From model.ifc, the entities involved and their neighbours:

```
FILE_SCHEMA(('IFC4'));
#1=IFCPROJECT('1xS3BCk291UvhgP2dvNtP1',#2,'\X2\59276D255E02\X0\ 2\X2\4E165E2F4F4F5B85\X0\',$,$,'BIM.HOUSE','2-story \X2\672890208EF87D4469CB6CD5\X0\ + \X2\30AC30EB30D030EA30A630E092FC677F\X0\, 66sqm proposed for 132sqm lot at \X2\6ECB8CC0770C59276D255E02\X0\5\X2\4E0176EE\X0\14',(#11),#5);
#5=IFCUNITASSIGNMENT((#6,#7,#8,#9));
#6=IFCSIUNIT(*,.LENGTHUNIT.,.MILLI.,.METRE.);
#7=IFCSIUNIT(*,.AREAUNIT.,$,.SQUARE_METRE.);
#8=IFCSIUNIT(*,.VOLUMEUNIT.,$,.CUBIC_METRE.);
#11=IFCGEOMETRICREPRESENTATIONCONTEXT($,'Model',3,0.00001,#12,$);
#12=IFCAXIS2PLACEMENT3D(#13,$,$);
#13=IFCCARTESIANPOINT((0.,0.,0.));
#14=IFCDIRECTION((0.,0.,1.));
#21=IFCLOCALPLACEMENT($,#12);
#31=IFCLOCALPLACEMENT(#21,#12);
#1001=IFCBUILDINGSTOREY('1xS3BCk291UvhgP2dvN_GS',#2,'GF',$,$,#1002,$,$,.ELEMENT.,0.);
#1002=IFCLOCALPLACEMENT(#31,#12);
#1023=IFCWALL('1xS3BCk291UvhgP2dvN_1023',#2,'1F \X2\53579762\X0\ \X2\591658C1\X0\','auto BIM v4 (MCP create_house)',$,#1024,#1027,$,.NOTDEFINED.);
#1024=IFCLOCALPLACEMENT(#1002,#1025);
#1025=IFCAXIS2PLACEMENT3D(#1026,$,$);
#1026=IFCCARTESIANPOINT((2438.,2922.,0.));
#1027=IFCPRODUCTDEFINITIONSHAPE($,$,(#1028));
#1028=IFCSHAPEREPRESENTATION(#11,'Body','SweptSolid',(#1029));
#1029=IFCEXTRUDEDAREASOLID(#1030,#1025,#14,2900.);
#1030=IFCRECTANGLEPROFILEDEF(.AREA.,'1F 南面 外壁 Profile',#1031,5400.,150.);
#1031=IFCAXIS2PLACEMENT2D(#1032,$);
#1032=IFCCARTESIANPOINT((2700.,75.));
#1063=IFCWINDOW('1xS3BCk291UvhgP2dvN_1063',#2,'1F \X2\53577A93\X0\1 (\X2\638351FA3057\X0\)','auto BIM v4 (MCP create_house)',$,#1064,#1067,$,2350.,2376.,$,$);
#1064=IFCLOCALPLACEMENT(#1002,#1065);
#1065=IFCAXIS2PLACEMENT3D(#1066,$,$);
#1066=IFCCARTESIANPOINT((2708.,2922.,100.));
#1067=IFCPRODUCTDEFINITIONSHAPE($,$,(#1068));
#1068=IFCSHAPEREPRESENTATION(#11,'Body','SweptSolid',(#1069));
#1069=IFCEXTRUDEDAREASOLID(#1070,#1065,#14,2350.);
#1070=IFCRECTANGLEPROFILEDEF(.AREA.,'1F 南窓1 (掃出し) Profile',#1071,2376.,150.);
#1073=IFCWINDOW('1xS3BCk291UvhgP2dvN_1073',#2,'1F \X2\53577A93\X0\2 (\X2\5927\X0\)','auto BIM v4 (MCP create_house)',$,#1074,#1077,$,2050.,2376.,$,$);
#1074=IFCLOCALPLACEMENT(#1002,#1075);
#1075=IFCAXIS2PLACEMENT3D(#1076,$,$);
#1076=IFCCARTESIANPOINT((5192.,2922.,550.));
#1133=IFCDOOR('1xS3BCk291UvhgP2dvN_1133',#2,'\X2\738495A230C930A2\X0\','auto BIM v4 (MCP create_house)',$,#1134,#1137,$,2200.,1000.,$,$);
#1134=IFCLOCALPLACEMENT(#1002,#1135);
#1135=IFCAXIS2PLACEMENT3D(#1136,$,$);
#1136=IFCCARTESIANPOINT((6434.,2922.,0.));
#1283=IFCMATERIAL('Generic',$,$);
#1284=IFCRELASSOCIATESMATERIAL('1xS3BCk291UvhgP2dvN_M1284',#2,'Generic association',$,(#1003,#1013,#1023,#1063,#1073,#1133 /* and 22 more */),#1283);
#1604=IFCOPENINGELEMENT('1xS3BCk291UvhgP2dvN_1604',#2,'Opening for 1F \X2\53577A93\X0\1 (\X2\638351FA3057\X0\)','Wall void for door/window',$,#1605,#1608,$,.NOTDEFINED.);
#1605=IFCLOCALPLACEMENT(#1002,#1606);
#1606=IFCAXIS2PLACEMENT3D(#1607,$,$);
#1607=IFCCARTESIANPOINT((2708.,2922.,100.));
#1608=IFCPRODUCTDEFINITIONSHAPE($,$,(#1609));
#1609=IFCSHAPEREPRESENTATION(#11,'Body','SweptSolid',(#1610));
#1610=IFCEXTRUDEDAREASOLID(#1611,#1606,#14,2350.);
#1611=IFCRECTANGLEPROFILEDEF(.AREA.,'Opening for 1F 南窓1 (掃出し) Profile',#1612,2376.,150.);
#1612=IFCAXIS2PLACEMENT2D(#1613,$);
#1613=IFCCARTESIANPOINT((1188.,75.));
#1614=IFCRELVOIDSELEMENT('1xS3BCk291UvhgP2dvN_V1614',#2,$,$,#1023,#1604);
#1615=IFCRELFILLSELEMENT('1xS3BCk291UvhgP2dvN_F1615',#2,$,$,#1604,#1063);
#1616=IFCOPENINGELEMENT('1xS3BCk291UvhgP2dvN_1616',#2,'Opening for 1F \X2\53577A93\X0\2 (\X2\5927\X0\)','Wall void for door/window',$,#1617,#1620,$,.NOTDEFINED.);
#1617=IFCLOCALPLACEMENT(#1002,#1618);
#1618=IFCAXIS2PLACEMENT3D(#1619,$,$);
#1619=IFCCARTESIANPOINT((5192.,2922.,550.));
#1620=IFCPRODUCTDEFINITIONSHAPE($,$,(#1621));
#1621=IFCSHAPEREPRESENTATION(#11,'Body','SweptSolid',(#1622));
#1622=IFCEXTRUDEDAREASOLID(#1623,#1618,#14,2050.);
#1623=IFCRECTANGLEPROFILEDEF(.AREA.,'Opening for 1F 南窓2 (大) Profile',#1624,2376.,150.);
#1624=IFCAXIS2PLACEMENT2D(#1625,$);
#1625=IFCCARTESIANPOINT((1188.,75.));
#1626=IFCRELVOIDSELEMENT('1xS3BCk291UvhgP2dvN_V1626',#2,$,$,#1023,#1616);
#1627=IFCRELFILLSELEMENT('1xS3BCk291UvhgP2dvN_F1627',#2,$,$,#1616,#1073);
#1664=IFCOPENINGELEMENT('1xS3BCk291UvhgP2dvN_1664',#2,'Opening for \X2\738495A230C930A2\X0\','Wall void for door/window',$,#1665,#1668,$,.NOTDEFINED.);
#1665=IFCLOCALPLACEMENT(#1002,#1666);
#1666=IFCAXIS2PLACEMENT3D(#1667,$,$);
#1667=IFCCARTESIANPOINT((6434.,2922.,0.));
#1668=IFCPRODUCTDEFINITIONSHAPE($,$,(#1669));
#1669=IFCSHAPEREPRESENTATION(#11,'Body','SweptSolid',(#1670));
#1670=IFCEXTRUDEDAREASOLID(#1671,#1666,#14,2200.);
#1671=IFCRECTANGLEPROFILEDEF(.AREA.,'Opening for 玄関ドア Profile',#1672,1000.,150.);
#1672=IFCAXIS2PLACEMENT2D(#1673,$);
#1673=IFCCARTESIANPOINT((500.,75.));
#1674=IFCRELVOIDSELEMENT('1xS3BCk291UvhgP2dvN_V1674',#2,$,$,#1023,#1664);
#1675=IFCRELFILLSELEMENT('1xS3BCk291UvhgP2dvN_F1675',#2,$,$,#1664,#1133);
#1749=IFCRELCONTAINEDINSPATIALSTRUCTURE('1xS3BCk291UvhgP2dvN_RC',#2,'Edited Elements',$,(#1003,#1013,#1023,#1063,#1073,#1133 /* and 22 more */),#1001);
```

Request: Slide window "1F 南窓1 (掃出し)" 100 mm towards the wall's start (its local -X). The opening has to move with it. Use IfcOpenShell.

```python
import ifcopenshell
import ifcopenshell.api.geometry
import ifcopenshell.util.placement
import ifcopenshell.util.unit

model = ifcopenshell.open("model.ifc")
unit_scale = ifcopenshell.util.unit.calculate_unit_scale(model)

window = model.by_id(1063)
opening = window.FillsVoids[0].RelatingOpeningElement
wall = opening.VoidsElements[0].RelatingBuildingElement

wall_matrix = ifcopenshell.util.placement.get_local_placement(wall.ObjectPlacement)
shift = wall_matrix[:3, 0] * -0.1 / unit_scale
before = ifcopenshell.util.placement.get_local_placement(window.ObjectPlacement)[:3, 3].copy()

# The window is not placed relative to its opening, so move both.
for product in (opening, window):
    matrix = ifcopenshell.util.placement.get_local_placement(product.ObjectPlacement)
    matrix[:3, 3] += shift
    ifcopenshell.api.geometry.edit_object_placement(model, product=product, matrix=matrix, is_si=False)

after = ifcopenshell.util.placement.get_local_placement(window.ObjectPlacement)[:3, 3]
print("window moved by", (after - before).round(3) + 0.0)

model.write("model_v2.ifc")
```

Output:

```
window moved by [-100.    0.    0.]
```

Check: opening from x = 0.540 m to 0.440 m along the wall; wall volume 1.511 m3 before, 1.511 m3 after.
